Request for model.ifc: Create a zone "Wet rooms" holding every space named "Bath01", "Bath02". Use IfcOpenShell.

First a look at what the model holds.

```python
import ifcopenshell

model = ifcopenshell.open("model.ifc")
print(model.schema)
seen = {}
for space in model.by_type("IfcSpace"):
    seen[space.Name] = seen.get(space.Name, 0) + 1
for name, count in sorted(seen.items(), key=str):
    print(count, "x", name)
print("zones:", [z.Name for z in model.by_type("IfcZone")][:20])
```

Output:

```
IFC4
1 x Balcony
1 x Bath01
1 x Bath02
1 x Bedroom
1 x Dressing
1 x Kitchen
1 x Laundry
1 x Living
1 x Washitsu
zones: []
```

```python
import ifcopenshell
import ifcopenshell.api.group
import ifcopenshell.api.root

model = ifcopenshell.open("model.ifc")

names = {"Bath01", "Bath02"}
spaces = [s for s in model.by_type("IfcSpace") if s.Name in names]

zone = ifcopenshell.api.root.create_entity(model, ifc_class="IfcZone", name="Wet rooms")
ifcopenshell.api.group.assign_group(model, products=spaces, group=zone)
print(len(spaces), "spaces in", zone.Name)

model.write("model_rev.ifc")
```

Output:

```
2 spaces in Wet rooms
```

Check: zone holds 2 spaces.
